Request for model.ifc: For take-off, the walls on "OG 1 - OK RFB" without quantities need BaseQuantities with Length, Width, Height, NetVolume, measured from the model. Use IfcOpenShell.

First a look at what the model holds.

```python
import ifcopenshell
import ifcopenshell.util.element
import ifcopenshell.util.unit

model = ifcopenshell.open("model.ifc")
print(model.schema)
for unit_type in ("LENGTHUNIT", "AREAUNIT", "VOLUMEUNIT"):
    print(unit_type, ifcopenshell.util.unit.calculate_unit_scale(model, unit_type))
storey = next(s for s in model.by_type("IfcBuildingStorey") if s.Name == "OG 1 - OK RFB")
walls = [e for e in ifcopenshell.util.element.get_decomposition(storey) if e.is_a("IfcWall")]
for e in sorted(walls, key=lambda e: e.id()):
    print(e.id(), e.is_a(), e.Name, list(ifcopenshell.util.element.get_psets(e, qtos_only=True)), sep=" | ")
```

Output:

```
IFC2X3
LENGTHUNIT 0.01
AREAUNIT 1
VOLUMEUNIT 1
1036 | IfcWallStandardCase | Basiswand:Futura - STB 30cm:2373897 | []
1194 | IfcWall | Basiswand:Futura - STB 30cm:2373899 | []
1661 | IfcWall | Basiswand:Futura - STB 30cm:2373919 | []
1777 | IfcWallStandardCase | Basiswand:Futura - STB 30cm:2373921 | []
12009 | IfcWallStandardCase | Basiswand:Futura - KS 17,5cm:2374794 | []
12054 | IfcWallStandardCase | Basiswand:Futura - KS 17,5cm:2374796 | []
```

```python
import ifcopenshell
import ifcopenshell.api.pset
import ifcopenshell.geom
import ifcopenshell.util.element
import ifcopenshell.util.shape
import ifcopenshell.util.unit

model = ifcopenshell.open("model.ifc")
unit_scale = ifcopenshell.util.unit.calculate_unit_scale(model)
volume_scale = ifcopenshell.util.unit.calculate_unit_scale(model, "VOLUMEUNIT")
settings = ifcopenshell.geom.settings()

storey = next(s for s in model.by_type("IfcBuildingStorey") if s.Name == "OG 1 - OK RFB")
walls = [e for e in ifcopenshell.util.element.get_decomposition(storey) if e.is_a("IfcWall")]

for e in sorted(walls, key=lambda e: e.id()):
    if ifcopenshell.util.element.get_psets(e, qtos_only=True, should_inherit=False):
        continue
    # Geometry comes back in metres, in the element's own axes.
    shape = ifcopenshell.geom.create_shape(settings, e)
    values = {
        "Length": ifcopenshell.util.shape.get_x(shape.geometry) / unit_scale,
        "Width": ifcopenshell.util.shape.get_y(shape.geometry) / unit_scale,
        "Height": ifcopenshell.util.shape.get_z(shape.geometry) / unit_scale,
        "NetVolume": ifcopenshell.util.shape.get_volume(shape.geometry) / volume_scale,
    }
    qto = ifcopenshell.api.pset.add_qto(model, product=e, name="BaseQuantities")
    ifcopenshell.api.pset.edit_qto(model, qto=qto, properties=values)
    print(e.id(), {k: round(v, 3) for k, v in values.items()})

model.write("model-out.ifc")
```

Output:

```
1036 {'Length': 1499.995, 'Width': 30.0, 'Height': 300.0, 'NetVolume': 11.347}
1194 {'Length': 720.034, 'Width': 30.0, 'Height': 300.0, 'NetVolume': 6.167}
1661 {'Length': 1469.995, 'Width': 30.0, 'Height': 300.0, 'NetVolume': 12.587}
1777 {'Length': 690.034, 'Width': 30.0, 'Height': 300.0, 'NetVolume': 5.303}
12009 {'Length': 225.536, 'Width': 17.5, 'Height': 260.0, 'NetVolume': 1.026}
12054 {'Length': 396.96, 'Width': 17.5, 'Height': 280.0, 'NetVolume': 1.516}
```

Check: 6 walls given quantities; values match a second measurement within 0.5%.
